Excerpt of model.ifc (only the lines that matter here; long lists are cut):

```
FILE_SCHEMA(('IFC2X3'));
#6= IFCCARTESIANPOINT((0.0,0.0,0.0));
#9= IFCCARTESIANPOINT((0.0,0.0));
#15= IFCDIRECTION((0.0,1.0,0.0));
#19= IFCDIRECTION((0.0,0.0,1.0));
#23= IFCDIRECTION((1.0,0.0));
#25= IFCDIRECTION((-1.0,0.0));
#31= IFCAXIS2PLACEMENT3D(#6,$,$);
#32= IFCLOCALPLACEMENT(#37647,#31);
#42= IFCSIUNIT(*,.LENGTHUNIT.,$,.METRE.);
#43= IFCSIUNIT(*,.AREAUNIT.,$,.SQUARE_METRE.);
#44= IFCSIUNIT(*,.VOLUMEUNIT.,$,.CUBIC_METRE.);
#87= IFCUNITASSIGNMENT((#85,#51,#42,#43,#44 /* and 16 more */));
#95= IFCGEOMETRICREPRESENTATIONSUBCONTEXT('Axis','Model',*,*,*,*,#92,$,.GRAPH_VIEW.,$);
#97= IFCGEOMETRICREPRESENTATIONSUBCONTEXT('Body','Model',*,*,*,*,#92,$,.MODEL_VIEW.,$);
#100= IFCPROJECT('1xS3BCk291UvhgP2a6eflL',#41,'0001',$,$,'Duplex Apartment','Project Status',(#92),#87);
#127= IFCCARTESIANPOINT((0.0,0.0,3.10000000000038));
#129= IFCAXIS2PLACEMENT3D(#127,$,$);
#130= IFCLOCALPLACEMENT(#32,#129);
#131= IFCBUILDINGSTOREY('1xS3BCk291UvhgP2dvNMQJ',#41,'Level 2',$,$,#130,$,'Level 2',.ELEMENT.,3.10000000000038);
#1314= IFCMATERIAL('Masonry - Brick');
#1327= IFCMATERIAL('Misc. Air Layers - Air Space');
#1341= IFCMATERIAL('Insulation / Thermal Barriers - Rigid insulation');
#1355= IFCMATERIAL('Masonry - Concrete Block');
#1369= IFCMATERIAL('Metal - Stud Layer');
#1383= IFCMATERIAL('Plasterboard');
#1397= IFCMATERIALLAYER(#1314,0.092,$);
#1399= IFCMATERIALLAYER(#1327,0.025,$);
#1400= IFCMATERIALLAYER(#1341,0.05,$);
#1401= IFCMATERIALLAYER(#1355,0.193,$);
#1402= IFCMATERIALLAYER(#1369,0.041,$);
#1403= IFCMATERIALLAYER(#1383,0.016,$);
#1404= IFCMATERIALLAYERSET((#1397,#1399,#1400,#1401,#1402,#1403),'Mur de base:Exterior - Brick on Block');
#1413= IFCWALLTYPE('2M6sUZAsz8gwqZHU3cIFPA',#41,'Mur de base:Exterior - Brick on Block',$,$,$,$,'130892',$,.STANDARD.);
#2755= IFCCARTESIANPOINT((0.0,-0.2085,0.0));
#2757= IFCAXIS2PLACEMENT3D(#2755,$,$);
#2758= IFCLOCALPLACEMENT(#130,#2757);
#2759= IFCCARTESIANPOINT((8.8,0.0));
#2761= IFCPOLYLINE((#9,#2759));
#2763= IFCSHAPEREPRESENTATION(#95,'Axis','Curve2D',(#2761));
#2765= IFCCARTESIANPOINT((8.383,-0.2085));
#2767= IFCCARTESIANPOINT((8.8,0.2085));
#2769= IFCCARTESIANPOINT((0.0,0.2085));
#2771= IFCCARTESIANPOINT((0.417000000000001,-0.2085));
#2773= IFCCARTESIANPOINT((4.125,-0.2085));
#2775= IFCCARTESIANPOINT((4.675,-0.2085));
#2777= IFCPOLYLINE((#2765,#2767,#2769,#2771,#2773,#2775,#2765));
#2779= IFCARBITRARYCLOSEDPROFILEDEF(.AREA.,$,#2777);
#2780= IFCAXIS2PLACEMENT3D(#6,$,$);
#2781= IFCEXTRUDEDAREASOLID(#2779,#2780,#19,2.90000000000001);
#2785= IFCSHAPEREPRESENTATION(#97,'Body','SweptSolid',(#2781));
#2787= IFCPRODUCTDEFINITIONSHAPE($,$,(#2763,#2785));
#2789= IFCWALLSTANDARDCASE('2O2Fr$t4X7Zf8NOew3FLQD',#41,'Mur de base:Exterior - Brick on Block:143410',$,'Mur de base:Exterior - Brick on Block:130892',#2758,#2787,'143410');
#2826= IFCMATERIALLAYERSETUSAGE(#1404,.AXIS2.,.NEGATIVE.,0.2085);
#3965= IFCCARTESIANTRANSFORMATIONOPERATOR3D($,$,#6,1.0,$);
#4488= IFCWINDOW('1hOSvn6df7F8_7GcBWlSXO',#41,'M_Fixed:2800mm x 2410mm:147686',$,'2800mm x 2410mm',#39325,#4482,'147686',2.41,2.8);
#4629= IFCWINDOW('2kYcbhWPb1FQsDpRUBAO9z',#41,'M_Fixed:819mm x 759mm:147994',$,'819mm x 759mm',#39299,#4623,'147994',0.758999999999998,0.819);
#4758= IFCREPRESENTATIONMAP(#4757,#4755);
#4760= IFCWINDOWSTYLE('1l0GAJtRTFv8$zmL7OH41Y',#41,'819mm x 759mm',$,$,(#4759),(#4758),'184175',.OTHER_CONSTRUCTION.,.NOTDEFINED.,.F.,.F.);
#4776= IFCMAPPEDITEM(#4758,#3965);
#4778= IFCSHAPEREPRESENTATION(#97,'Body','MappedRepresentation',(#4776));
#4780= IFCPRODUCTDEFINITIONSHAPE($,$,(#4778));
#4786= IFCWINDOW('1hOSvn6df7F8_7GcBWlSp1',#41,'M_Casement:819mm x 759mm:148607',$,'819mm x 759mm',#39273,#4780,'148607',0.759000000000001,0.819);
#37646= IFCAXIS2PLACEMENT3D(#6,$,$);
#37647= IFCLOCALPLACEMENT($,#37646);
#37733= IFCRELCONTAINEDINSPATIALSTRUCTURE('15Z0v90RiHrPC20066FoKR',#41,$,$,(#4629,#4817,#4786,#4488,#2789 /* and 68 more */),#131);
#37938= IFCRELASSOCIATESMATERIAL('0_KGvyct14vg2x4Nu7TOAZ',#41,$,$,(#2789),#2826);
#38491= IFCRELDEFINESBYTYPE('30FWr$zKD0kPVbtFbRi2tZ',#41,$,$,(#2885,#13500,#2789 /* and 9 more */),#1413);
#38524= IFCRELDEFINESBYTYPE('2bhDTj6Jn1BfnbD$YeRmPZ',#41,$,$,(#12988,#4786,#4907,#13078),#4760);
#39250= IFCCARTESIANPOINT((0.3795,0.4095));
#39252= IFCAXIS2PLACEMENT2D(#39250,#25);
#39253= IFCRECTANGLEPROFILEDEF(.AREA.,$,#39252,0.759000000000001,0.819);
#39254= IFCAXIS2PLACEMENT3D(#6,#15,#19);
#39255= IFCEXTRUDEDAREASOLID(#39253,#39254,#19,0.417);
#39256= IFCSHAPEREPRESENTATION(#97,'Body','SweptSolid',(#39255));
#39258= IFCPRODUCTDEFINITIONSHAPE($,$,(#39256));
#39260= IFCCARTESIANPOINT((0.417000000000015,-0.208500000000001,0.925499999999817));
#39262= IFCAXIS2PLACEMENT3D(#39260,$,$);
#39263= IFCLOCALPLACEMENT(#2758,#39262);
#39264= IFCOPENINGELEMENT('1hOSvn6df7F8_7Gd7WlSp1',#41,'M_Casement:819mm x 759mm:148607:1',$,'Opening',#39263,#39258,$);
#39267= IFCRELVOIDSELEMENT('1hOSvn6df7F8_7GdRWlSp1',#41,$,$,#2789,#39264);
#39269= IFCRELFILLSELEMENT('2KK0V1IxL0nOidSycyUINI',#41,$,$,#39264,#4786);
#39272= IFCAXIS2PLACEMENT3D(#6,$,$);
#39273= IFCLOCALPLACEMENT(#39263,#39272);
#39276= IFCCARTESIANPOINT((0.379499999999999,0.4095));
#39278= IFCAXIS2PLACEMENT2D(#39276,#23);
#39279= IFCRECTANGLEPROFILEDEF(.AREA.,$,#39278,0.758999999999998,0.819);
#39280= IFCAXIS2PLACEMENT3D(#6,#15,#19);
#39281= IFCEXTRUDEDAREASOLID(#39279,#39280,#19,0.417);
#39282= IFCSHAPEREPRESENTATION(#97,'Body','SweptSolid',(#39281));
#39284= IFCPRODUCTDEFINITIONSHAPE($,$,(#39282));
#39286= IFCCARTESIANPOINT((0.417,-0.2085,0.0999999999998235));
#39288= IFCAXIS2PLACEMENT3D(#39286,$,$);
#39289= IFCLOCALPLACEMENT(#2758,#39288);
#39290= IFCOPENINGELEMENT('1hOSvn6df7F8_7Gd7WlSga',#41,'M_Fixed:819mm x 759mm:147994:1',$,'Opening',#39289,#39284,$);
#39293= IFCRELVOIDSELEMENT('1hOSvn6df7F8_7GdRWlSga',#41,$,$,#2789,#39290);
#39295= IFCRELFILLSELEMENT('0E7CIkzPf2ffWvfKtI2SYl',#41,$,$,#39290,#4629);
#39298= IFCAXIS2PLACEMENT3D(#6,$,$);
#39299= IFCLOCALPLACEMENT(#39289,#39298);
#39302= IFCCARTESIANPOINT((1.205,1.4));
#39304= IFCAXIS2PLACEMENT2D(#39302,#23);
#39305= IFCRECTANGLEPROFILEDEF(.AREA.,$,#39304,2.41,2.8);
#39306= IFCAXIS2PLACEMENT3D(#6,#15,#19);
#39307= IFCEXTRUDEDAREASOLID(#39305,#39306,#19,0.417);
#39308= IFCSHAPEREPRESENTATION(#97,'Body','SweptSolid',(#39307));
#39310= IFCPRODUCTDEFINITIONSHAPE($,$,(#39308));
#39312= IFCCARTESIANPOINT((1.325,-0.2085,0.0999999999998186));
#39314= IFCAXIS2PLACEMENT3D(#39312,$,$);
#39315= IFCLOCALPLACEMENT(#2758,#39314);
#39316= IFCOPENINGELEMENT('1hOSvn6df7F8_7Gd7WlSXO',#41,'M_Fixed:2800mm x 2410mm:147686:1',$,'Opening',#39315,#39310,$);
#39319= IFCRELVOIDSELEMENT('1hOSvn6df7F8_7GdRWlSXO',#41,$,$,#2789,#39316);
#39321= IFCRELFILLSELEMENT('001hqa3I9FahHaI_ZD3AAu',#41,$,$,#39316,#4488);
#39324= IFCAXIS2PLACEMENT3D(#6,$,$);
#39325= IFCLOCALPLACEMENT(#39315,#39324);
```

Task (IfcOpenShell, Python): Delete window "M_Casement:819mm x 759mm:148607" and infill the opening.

```python
import ifcopenshell
import ifcopenshell.api.feature
import ifcopenshell.api.root
import ifcopenshell.geom
import ifcopenshell.util.shape

model = ifcopenshell.open("model.ifc")
settings = ifcopenshell.geom.settings()


def volume(element):
    """Net volume in cubic metres, openings subtracted."""
    shape = ifcopenshell.geom.create_shape(settings, element)
    return ifcopenshell.util.shape.get_volume(shape.geometry)


window = model.by_guid("1hOSvn6df7F8_7GcBWlSp1")
opening = window.FillsVoids[0].RelatingOpeningElement
wall = opening.VoidsElements[0].RelatingBuildingElement
before = volume(wall)

ifcopenshell.api.root.remove_product(model, product=window)
ifcopenshell.api.feature.remove_feature(model, feature=opening)

after = volume(wall)

print(f"wall volume {before:.3f} -> {after:.3f} m3")

model.write("model_updated.ifc")
```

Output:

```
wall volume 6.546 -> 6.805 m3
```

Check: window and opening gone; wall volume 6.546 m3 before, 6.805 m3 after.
